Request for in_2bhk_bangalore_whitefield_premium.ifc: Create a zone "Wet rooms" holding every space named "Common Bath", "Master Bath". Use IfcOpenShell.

First a look at what the model holds.

```python
import ifcopenshell

model = ifcopenshell.open("in_2bhk_bangalore_whitefield_premium.ifc")
print(model.schema)
seen = {}
for space in model.by_type("IfcSpace"):
    seen[space.LongName] = seen.get(space.LongName, 0) + 1
for name, count in sorted(seen.items(), key=str):
    print(count, "x", name)
print("zones:", [z.Name for z in model.by_type("IfcZone")][:20])
```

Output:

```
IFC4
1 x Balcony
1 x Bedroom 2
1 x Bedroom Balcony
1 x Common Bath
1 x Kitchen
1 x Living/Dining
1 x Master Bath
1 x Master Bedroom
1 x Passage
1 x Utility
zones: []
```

```python
import ifcopenshell
import ifcopenshell.api.group
import ifcopenshell.api.root

model = ifcopenshell.open("in_2bhk_bangalore_whitefield_premium.ifc")

names = {"Common Bath", "Master Bath"}
spaces = [s for s in model.by_type("IfcSpace") if s.LongName in names]

zone = ifcopenshell.api.root.create_entity(model, ifc_class="IfcZone", name="Wet rooms")
ifcopenshell.api.group.assign_group(model, products=spaces, group=zone)
print(len(spaces), "spaces in", zone.Name)

model.write("in_2bhk_bangalore_whitefield_premium_edited.ifc")
```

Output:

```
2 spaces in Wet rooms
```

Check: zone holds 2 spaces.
